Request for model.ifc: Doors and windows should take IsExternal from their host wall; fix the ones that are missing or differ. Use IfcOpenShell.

First a look at what the model holds.

```python
import ifcopenshell
import ifcopenshell.util.element

model = ifcopenshell.open("model.ifc")
print(model.schema)
seen = {}
for e in model.by_type("IfcDoor") + model.by_type("IfcWindow"):
    if not e.FillsVoids:
        continue
    host = e.FillsVoids[0].RelatingOpeningElement.VoidsElements[0].RelatingBuildingElement
    own = ifcopenshell.util.element.get_pset(e, f"Pset_{e.is_a()[3:].removesuffix('StandardCase')}Common", "IsExternal")
    wall = ifcopenshell.util.element.get_pset(host, "Pset_WallCommon", "IsExternal")
    seen[e.is_a(), own, wall] = seen.get((e.is_a(), own, wall), 0) + 1
for (cls, own, wall), count in sorted(seen.items(), key=str):
    print(count, cls, "IsExternal:", own, "| host wall:", wall)
```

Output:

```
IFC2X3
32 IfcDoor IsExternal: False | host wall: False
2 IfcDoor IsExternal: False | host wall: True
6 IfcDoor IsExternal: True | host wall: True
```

```python
import ifcopenshell
import ifcopenshell.api.pset
import ifcopenshell.util.element

model = ifcopenshell.open("model.ifc")

count = 0
for ifc_class, pset_name in (("IfcDoor", "Pset_DoorCommon"), ("IfcWindow", "Pset_WindowCommon")):
    for e in model.by_type(ifc_class):
        if not e.FillsVoids:
            continue
        host = e.FillsVoids[0].RelatingOpeningElement.VoidsElements[0].RelatingBuildingElement
        external = ifcopenshell.util.element.get_pset(host, "Pset_WallCommon", "IsExternal")
        if external is None or ifcopenshell.util.element.get_pset(e, pset_name, "IsExternal") == external:
            continue
        pset = ifcopenshell.api.pset.add_pset(model, product=e, name=pset_name)
        ifcopenshell.api.pset.edit_pset(model, pset=pset, properties={"IsExternal": external})
        count += 1

print(count, "updated")

model.write("model_rev.ifc")
```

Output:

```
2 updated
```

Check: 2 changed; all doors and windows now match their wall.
